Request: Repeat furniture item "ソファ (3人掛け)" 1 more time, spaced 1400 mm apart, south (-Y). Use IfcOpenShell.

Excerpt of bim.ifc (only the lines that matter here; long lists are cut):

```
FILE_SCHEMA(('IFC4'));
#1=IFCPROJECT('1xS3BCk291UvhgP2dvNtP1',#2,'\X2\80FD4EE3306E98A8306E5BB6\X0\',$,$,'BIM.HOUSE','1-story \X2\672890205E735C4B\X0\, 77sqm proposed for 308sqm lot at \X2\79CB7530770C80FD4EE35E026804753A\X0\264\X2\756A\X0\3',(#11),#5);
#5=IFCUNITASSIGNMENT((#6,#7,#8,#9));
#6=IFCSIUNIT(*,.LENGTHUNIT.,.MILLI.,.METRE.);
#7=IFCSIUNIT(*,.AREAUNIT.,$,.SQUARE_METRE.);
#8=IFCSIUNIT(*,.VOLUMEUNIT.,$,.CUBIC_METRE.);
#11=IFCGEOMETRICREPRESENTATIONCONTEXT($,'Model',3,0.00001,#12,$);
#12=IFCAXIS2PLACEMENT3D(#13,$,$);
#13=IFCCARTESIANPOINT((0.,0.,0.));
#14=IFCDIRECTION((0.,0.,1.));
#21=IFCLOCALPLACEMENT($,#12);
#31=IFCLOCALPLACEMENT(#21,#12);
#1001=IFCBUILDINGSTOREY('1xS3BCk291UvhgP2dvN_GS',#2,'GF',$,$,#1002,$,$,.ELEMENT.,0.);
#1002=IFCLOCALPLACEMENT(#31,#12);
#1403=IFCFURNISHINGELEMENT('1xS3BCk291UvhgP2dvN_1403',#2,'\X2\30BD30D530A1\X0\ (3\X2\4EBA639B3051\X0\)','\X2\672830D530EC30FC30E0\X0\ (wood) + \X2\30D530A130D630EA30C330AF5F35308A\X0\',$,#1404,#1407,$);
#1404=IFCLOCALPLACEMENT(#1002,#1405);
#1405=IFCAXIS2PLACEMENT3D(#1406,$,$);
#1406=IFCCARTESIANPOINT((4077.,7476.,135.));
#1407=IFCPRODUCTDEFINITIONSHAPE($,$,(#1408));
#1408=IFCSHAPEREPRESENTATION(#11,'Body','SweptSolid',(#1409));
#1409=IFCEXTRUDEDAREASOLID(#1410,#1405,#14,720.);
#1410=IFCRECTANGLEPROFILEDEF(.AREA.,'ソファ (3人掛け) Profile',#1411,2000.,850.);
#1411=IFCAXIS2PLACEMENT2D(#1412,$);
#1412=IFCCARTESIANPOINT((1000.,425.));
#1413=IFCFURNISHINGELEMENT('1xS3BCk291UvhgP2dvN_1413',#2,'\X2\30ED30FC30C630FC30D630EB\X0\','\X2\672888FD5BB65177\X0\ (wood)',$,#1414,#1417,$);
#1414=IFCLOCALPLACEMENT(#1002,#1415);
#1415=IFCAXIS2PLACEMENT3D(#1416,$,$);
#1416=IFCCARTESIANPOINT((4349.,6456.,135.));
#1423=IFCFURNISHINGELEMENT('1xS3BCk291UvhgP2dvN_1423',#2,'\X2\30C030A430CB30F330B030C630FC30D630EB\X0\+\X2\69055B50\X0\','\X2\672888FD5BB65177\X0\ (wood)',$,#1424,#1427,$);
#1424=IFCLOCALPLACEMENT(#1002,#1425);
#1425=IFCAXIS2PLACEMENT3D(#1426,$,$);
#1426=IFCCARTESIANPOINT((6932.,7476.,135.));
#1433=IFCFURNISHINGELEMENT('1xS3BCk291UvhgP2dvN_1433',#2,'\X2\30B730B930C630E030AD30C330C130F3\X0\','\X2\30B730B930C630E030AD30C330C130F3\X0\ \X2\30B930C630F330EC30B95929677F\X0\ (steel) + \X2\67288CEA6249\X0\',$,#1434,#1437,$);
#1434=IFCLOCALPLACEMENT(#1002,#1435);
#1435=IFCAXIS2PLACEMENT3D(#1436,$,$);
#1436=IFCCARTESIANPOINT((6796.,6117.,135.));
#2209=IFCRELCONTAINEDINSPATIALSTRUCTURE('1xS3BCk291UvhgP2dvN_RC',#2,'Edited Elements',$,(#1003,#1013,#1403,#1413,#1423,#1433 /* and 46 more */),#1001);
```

```python
import numpy as np
import ifcopenshell
import ifcopenshell.api.geometry
import ifcopenshell.api.root
import ifcopenshell.util.element
import ifcopenshell.util.placement

model = ifcopenshell.open("bim.ifc")


def reuse_history(source, copy):
    """copy_class also copies each property set's owner history, people and application; keep the originals."""
    for rel in copy.IsDefinedBy:
        if rel.is_a("IfcRelDefinesByProperties") and (history := rel.RelatingPropertyDefinition.OwnerHistory):
            rel.RelatingPropertyDefinition.OwnerHistory = source.OwnerHistory
            ifcopenshell.util.element.remove_deep2(model, history)


source = model.by_guid("1xS3BCk291UvhgP2dvN_1403")
base = ifcopenshell.util.placement.get_local_placement(source.ObjectPlacement)
step = np.array([0.0, -1.0, 0.0]) * 1400.0

for i in range(1, 2):
    copy = ifcopenshell.api.root.copy_class(model, product=source)
    copy.Representation = ifcopenshell.util.element.copy_deep(
        model, source.Representation, exclude=["IfcGeometricRepresentationContext", "IfcRepresentationMap"]
    )
    reuse_history(source, copy)
    matrix = base.copy()
    matrix[:3, 3] += i * step
    print("added at", matrix[:3, 3].round(3) + 0.0)
    ifcopenshell.api.geometry.edit_object_placement(model, product=copy, matrix=matrix, is_si=False)

model.write("bim_rev.ifc")
```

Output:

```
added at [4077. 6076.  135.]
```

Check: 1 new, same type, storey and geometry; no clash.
